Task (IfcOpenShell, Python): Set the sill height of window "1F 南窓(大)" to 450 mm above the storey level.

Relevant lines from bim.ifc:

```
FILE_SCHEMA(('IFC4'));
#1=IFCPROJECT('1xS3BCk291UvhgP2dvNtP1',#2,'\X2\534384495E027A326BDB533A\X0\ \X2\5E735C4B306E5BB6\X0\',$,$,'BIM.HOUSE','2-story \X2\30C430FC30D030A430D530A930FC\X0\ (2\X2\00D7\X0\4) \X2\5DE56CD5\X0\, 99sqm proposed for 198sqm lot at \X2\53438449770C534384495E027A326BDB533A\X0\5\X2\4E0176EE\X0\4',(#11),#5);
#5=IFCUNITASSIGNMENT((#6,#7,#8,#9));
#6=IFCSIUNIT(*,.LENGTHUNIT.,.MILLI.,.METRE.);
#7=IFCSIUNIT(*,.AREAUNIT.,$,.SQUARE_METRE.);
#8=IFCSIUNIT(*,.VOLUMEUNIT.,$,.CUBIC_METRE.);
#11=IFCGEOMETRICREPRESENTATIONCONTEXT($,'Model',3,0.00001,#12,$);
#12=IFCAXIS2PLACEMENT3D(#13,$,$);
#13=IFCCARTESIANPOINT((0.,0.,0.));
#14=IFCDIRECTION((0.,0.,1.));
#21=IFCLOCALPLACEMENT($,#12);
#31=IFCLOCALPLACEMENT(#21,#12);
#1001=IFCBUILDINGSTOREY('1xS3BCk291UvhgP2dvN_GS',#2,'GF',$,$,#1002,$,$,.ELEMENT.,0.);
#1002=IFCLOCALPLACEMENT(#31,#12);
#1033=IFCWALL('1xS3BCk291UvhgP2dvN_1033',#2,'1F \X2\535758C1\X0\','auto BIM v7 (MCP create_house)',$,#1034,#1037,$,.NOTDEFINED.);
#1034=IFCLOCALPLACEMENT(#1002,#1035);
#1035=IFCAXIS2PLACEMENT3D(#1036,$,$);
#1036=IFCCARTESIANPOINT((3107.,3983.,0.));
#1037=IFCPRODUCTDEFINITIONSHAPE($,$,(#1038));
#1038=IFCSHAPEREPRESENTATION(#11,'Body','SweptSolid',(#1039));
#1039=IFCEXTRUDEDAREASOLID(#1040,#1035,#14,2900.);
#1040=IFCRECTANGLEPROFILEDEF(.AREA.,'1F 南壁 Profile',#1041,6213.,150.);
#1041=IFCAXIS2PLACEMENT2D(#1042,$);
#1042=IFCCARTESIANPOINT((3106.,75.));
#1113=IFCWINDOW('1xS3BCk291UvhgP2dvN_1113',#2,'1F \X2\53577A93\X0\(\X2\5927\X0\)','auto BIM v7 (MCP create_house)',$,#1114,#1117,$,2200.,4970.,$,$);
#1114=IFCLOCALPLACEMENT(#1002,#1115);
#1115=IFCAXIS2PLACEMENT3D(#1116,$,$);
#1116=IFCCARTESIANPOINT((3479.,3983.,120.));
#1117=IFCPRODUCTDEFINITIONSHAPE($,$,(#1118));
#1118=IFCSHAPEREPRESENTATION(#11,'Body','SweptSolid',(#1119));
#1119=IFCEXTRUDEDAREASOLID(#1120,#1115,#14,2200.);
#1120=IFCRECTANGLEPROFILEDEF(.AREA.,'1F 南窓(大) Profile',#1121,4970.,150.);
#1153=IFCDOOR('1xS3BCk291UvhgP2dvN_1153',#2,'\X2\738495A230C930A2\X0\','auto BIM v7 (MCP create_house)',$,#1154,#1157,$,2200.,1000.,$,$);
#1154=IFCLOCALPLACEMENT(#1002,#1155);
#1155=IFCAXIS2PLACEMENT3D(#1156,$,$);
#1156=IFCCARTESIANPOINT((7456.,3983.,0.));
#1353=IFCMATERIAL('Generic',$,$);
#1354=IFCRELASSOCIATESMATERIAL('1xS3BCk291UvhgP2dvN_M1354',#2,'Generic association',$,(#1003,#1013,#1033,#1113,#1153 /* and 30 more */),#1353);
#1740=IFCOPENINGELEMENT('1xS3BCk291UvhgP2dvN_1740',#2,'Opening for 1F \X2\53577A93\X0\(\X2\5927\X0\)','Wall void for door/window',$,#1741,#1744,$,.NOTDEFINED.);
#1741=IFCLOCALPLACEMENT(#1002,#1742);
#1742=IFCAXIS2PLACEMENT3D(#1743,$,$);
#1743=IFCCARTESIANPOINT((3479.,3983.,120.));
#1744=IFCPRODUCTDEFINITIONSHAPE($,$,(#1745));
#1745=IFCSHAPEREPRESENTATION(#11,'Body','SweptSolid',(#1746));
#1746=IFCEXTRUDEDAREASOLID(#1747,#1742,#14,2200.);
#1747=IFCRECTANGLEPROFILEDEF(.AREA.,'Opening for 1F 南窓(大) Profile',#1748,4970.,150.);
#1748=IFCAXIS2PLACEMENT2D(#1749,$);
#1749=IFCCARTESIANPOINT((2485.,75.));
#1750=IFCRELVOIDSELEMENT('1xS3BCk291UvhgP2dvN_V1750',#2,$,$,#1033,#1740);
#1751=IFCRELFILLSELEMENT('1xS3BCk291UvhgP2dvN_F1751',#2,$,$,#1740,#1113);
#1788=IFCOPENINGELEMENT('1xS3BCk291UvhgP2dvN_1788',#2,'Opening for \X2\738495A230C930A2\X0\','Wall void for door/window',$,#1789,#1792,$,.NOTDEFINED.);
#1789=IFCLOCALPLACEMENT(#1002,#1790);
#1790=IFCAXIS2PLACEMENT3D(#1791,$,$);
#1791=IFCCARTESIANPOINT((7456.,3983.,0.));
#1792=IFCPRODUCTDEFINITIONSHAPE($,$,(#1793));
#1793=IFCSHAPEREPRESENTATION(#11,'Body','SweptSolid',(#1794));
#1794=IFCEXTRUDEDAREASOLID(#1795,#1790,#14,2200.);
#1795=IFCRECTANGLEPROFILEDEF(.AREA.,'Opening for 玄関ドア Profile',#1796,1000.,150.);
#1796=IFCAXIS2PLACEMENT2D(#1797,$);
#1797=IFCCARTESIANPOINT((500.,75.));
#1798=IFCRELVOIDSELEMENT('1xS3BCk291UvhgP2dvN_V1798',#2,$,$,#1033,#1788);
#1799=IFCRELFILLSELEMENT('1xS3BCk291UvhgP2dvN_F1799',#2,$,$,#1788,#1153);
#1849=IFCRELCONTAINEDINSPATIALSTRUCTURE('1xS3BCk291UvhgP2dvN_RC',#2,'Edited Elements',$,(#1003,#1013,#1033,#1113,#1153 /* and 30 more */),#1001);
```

```python
import numpy as np
import ifcopenshell
import ifcopenshell.api.geometry
import ifcopenshell.geom
import ifcopenshell.util.element
import ifcopenshell.util.placement
import ifcopenshell.util.shape
import ifcopenshell.util.unit

model = ifcopenshell.open("bim.ifc")
unit_scale = ifcopenshell.util.unit.calculate_unit_scale(model)

window = model.by_guid("1xS3BCk291UvhgP2dvN_1113")
opening = window.FillsVoids[0].RelatingOpeningElement
storey = ifcopenshell.util.element.get_container(window, ifc_class="IfcBuildingStorey")
level = ifcopenshell.util.placement.get_local_placement(storey.ObjectPlacement)[2, 3]

# The opening's origin need not be at the sill, so measure its lowest point.
shape = ifcopenshell.geom.create_shape(ifcopenshell.geom.settings(), opening)
bottom = ifcopenshell.util.shape.get_shape_bottom_elevation(shape, shape.geometry) / unit_scale
dz = level + 0.45 / unit_scale - bottom

shift = np.array([0.0, 0.0, dz])
# The window is not placed relative to its opening, so move both.
for product in (opening, window):
    matrix = ifcopenshell.util.placement.get_local_placement(product.ObjectPlacement)
    matrix[:3, 3] += shift
    ifcopenshell.api.geometry.edit_object_placement(model, product=product, matrix=matrix, is_si=False)

print(f"moved by {dz * unit_scale:+.3f} m")

model.write("bim-out.ifc")
```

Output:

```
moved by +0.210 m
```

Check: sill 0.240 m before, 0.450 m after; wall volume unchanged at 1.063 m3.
